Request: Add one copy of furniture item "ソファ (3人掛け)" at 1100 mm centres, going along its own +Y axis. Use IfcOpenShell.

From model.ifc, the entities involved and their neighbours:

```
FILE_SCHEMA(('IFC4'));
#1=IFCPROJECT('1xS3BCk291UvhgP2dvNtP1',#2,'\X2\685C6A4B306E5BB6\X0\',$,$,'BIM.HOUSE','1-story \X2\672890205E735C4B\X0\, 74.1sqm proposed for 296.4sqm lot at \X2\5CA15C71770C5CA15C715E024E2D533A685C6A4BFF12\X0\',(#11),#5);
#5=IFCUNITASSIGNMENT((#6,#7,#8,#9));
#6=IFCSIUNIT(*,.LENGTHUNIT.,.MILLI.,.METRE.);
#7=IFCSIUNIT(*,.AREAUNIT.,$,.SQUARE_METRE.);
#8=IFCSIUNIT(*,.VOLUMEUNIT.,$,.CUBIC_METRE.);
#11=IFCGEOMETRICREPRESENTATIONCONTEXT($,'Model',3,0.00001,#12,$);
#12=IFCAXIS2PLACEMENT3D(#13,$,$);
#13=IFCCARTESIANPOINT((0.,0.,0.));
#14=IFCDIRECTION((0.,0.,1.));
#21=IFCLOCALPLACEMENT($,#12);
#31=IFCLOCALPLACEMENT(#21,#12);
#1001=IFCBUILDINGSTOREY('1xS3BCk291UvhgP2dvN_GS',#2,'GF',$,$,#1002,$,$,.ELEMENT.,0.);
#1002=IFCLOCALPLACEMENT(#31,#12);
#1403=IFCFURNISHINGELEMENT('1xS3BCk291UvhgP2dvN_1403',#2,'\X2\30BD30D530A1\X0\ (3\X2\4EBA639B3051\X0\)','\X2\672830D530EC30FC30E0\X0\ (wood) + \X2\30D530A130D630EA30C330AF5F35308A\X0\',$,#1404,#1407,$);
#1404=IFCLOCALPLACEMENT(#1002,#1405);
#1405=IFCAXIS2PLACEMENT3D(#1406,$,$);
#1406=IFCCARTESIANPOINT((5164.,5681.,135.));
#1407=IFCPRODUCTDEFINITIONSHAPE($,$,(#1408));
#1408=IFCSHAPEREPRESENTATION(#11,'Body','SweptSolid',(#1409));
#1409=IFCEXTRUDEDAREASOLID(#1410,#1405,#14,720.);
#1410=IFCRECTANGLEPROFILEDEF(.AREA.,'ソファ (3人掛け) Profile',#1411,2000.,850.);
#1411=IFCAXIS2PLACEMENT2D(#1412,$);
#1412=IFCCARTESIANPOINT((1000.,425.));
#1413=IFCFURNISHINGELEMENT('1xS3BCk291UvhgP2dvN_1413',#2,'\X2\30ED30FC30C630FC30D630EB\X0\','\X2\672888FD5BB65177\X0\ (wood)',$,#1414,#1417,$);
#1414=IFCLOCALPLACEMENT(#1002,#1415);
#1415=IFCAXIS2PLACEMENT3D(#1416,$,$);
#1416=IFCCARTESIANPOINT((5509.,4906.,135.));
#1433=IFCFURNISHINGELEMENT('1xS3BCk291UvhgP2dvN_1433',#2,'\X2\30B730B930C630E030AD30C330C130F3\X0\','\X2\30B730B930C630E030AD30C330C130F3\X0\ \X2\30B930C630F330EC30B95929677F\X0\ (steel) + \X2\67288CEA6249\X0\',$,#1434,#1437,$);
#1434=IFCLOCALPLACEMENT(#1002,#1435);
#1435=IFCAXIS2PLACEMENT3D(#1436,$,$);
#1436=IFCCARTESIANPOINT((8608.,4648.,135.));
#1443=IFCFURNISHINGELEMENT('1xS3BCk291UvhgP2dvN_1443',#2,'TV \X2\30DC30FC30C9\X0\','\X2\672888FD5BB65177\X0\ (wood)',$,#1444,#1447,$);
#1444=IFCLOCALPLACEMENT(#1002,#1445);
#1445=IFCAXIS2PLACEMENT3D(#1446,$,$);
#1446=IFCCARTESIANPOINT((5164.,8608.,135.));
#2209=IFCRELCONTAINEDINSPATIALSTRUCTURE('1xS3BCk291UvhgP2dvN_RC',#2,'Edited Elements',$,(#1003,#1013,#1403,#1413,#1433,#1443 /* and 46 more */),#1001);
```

```python
import ifcopenshell
import ifcopenshell.api.geometry
import ifcopenshell.api.root
import ifcopenshell.util.element
import ifcopenshell.util.placement
import ifcopenshell.util.unit

model = ifcopenshell.open("model.ifc")
unit_scale = ifcopenshell.util.unit.calculate_unit_scale(model)


def reuse_history(source, copy):
    """copy_class also copies each property set's owner history, people and application; keep the originals."""
    for rel in copy.IsDefinedBy:
        if rel.is_a("IfcRelDefinesByProperties") and (history := rel.RelatingPropertyDefinition.OwnerHistory):
            rel.RelatingPropertyDefinition.OwnerHistory = source.OwnerHistory
            ifcopenshell.util.element.remove_deep2(model, history)


source = model.by_guid("1xS3BCk291UvhgP2dvN_1403")
base = ifcopenshell.util.placement.get_local_placement(source.ObjectPlacement)
step = base[:3, 1] * 1.1 / unit_scale

for i in range(1, 2):
    copy = ifcopenshell.api.root.copy_class(model, product=source)
    copy.Representation = ifcopenshell.util.element.copy_deep(
        model, source.Representation, exclude=["IfcGeometricRepresentationContext", "IfcRepresentationMap"]
    )
    reuse_history(source, copy)
    matrix = base.copy()
    matrix[:3, 3] += i * step
    print("added at", matrix[:3, 3].round(3) + 0.0)
    ifcopenshell.api.geometry.edit_object_placement(model, product=copy, matrix=matrix, is_si=False)

model.write("model_v2.ifc")
```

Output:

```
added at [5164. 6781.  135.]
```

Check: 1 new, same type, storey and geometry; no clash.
